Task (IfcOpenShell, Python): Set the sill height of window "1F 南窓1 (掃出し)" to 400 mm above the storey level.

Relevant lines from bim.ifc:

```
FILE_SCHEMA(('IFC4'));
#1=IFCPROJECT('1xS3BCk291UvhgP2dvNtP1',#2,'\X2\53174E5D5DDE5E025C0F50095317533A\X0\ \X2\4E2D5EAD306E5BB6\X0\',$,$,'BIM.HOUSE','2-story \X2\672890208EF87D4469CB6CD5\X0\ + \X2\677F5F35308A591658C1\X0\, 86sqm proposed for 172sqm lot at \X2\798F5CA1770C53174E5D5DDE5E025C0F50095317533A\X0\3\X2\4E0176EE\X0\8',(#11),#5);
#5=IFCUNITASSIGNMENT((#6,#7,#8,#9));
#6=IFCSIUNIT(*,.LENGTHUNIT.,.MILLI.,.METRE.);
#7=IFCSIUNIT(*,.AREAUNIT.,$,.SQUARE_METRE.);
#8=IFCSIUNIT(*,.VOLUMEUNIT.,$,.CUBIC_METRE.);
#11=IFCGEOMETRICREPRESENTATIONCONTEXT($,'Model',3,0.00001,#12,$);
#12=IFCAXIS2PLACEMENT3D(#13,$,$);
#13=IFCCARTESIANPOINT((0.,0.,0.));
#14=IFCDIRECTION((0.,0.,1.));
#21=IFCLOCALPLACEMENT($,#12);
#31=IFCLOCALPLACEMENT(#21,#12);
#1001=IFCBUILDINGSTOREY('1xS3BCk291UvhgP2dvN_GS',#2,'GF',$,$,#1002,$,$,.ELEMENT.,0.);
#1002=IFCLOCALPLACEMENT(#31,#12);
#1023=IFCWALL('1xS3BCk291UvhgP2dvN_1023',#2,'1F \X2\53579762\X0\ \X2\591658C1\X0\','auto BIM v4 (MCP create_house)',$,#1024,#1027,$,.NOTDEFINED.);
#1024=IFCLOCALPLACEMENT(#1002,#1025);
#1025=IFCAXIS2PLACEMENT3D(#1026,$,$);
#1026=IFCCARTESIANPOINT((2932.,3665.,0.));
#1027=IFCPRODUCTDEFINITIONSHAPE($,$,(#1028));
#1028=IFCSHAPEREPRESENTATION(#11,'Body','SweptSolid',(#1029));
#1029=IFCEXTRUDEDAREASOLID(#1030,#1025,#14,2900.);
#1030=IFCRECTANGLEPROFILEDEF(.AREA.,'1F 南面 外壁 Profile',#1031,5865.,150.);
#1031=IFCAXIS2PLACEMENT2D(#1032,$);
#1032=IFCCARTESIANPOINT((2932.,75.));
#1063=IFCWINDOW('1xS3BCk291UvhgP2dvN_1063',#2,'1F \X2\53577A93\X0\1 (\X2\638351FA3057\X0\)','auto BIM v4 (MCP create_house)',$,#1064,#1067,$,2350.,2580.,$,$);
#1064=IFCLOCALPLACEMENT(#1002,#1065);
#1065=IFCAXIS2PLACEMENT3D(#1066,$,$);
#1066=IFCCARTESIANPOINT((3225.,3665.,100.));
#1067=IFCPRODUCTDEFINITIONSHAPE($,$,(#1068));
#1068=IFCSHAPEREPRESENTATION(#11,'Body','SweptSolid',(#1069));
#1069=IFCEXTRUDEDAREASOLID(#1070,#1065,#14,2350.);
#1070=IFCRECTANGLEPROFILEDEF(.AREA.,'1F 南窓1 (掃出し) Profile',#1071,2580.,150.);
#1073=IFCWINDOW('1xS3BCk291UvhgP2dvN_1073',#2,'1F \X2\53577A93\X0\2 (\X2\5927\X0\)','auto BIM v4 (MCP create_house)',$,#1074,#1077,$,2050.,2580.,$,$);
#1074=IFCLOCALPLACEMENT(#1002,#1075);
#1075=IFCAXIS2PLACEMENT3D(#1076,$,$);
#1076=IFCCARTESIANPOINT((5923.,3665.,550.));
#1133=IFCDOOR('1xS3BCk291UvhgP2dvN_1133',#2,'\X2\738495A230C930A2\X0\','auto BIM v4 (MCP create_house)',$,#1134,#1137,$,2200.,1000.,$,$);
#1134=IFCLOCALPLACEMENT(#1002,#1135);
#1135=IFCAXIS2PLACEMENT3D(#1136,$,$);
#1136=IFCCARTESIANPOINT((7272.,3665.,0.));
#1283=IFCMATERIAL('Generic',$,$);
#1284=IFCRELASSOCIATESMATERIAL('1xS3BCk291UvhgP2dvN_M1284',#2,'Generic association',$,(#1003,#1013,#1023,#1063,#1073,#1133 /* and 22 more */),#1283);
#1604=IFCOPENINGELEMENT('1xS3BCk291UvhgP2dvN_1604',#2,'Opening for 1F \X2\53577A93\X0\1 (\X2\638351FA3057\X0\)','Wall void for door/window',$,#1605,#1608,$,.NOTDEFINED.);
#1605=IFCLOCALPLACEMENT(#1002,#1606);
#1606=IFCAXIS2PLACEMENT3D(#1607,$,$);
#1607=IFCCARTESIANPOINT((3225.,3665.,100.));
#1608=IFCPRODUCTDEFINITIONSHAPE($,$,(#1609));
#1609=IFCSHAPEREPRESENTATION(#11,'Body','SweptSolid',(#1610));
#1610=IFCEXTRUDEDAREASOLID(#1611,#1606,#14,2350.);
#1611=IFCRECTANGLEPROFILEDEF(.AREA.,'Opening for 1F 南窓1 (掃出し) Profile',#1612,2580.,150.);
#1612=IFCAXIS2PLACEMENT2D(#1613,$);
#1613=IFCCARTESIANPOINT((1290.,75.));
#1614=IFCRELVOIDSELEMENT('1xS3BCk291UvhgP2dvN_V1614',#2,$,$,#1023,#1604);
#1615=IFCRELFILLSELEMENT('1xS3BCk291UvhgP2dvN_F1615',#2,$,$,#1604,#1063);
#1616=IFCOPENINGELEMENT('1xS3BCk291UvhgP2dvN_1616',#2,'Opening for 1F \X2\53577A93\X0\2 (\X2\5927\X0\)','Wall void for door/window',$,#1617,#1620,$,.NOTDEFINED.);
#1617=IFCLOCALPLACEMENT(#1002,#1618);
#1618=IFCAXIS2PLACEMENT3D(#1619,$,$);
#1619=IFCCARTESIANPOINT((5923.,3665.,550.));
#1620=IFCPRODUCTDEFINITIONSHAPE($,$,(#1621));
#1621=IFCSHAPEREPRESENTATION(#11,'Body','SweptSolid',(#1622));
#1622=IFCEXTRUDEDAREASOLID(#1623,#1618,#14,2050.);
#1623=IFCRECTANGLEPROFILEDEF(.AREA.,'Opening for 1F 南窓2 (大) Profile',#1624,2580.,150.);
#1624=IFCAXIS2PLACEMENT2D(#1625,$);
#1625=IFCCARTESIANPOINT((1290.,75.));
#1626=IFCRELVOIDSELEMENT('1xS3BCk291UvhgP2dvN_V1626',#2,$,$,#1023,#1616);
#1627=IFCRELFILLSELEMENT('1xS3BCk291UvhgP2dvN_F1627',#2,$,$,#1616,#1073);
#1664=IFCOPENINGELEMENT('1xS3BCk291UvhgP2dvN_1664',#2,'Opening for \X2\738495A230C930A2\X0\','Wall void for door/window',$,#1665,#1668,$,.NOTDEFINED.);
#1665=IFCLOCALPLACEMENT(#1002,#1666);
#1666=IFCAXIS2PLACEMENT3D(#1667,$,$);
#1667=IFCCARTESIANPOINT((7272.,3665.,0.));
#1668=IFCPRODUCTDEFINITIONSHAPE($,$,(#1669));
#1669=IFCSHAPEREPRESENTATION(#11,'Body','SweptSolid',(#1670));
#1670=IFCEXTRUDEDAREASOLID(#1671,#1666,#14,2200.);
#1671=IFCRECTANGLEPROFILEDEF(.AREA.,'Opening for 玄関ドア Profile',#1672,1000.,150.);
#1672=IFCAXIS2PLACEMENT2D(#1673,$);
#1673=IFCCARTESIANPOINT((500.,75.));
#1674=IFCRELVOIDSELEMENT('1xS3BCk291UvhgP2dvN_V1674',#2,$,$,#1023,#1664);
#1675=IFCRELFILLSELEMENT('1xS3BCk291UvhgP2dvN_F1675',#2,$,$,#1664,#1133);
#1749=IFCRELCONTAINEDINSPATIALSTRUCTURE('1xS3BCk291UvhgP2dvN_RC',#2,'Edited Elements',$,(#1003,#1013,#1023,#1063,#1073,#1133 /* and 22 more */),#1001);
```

```python
import numpy as np
import ifcopenshell
import ifcopenshell.api.geometry
import ifcopenshell.geom
import ifcopenshell.util.element
import ifcopenshell.util.placement
import ifcopenshell.util.shape
import ifcopenshell.util.unit

model = ifcopenshell.open("bim.ifc")
unit_scale = ifcopenshell.util.unit.calculate_unit_scale(model)

window = model.by_guid("1xS3BCk291UvhgP2dvN_1063")
opening = window.FillsVoids[0].RelatingOpeningElement
storey = ifcopenshell.util.element.get_container(window, ifc_class="IfcBuildingStorey")
level = ifcopenshell.util.placement.get_local_placement(storey.ObjectPlacement)[2, 3]

# The opening's origin need not be at the sill, so measure its lowest point.
shape = ifcopenshell.geom.create_shape(ifcopenshell.geom.settings(), opening)
bottom = ifcopenshell.util.shape.get_shape_bottom_elevation(shape, shape.geometry) / unit_scale
dz = level + 0.4 / unit_scale - bottom

shift = np.array([0.0, 0.0, dz])
# The window is not placed relative to its opening, so move both.
for product in (opening, window):
    matrix = ifcopenshell.util.placement.get_local_placement(product.ObjectPlacement)
    matrix[:3, 3] += shift
    ifcopenshell.api.geometry.edit_object_placement(model, product=product, matrix=matrix, is_si=False)

print(f"moved by {dz * unit_scale:+.3f} m")

model.write("bim-out.ifc")
```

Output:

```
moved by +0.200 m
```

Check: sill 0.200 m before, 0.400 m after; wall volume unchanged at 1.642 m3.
